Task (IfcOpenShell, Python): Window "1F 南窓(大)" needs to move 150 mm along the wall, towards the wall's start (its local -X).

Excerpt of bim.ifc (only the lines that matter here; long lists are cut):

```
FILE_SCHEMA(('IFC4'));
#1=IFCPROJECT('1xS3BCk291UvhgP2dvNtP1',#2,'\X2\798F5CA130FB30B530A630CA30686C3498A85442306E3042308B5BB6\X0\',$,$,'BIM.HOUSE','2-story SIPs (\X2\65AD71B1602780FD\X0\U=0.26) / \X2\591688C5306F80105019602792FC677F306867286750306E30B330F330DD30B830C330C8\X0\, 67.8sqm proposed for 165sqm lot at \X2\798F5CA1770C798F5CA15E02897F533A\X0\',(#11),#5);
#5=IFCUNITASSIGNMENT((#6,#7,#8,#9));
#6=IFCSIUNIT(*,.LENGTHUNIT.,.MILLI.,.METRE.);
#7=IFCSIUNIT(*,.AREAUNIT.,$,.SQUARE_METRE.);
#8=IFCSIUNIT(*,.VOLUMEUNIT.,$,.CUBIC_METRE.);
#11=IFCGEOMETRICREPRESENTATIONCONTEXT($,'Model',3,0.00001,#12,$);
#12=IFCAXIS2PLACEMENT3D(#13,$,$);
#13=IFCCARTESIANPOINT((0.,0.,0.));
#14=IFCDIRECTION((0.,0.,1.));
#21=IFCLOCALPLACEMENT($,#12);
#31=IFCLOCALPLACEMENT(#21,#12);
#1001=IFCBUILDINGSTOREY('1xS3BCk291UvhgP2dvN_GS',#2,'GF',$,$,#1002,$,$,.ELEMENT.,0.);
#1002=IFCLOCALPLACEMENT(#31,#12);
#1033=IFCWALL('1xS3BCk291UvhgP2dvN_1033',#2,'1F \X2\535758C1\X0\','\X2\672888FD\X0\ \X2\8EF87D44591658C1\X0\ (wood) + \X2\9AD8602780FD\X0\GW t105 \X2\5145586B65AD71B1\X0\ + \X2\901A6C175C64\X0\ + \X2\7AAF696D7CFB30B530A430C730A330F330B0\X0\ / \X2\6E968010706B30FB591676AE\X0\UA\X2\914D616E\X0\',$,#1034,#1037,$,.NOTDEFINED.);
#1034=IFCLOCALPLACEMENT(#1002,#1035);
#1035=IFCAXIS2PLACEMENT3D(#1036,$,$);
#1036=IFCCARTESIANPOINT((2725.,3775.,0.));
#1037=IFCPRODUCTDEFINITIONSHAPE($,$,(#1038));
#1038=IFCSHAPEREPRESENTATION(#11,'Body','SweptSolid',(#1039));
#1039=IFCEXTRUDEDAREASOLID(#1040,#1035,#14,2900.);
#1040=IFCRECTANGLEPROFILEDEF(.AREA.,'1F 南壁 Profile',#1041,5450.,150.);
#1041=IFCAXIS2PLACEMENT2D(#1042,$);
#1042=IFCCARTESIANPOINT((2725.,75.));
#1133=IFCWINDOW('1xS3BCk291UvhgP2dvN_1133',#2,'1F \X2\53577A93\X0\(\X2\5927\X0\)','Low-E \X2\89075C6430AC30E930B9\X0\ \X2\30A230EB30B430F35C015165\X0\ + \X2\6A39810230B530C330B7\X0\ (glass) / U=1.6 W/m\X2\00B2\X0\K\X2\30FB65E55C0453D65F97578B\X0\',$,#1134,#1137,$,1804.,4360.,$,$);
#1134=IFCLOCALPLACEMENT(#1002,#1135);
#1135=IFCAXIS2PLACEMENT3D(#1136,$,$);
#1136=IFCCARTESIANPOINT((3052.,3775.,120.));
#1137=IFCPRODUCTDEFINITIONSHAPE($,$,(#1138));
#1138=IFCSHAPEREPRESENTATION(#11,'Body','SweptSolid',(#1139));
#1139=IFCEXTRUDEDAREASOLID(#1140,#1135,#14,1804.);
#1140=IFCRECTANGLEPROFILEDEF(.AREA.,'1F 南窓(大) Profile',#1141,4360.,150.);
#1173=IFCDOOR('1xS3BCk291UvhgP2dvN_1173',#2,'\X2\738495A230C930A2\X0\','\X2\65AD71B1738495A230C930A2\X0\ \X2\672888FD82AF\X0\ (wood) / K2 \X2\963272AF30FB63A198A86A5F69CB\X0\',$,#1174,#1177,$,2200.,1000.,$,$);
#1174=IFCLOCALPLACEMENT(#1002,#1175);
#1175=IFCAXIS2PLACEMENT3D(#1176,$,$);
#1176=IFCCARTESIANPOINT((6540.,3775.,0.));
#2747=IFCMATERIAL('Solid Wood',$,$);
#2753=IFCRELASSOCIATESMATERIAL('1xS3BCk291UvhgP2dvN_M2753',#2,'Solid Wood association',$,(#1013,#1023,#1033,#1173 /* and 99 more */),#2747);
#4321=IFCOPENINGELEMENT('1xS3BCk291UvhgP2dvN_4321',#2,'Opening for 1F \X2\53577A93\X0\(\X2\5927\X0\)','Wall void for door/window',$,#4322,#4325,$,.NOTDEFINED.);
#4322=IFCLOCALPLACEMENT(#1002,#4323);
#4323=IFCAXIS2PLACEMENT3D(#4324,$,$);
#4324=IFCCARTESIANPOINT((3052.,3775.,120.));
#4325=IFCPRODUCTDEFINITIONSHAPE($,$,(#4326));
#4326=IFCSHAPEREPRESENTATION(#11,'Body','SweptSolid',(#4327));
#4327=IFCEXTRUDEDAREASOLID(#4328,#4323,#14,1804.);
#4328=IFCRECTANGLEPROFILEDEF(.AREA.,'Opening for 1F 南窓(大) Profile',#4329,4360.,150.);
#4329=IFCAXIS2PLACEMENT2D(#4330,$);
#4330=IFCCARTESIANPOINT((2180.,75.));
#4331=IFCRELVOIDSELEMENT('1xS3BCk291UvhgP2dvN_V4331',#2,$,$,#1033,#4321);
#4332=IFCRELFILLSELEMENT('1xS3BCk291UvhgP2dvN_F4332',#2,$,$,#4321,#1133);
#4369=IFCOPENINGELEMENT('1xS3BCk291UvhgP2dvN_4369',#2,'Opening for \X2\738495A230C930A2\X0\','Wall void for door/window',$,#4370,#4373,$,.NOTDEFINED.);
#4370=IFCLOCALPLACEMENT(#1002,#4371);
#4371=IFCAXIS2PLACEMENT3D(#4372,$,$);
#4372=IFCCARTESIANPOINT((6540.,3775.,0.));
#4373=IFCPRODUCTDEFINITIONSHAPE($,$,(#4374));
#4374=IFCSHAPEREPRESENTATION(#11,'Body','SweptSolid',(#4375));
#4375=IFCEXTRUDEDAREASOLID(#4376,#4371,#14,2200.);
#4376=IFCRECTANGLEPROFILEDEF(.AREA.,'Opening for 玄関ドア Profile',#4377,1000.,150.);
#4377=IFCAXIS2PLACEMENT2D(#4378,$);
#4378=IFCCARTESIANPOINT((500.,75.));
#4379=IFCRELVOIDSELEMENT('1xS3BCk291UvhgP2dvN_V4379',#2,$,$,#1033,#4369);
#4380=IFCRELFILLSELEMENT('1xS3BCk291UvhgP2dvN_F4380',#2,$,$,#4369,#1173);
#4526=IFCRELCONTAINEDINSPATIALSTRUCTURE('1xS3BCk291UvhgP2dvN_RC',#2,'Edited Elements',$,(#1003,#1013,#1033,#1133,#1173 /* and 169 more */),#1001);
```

```python
import ifcopenshell
import ifcopenshell.api.geometry
import ifcopenshell.util.placement
import ifcopenshell.util.unit

model = ifcopenshell.open("bim.ifc")
unit_scale = ifcopenshell.util.unit.calculate_unit_scale(model)

window = model.by_guid("1xS3BCk291UvhgP2dvN_1133")
opening = window.FillsVoids[0].RelatingOpeningElement
wall = opening.VoidsElements[0].RelatingBuildingElement

wall_matrix = ifcopenshell.util.placement.get_local_placement(wall.ObjectPlacement)
shift = wall_matrix[:3, 0] * -0.15 / unit_scale
before = ifcopenshell.util.placement.get_local_placement(window.ObjectPlacement)[:3, 3].copy()

# The window is not placed relative to its opening, so move both.
for product in (opening, window):
    matrix = ifcopenshell.util.placement.get_local_placement(product.ObjectPlacement)
    matrix[:3, 3] += shift
    ifcopenshell.api.geometry.edit_object_placement(model, product=product, matrix=matrix, is_si=False)

after = ifcopenshell.util.placement.get_local_placement(window.ObjectPlacement)[:3, 3]
print("window moved by", (after - before).round(3) + 0.0)

model.write("bim_updated.ifc")
```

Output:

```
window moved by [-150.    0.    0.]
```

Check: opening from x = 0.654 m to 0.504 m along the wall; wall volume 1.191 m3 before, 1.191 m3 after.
